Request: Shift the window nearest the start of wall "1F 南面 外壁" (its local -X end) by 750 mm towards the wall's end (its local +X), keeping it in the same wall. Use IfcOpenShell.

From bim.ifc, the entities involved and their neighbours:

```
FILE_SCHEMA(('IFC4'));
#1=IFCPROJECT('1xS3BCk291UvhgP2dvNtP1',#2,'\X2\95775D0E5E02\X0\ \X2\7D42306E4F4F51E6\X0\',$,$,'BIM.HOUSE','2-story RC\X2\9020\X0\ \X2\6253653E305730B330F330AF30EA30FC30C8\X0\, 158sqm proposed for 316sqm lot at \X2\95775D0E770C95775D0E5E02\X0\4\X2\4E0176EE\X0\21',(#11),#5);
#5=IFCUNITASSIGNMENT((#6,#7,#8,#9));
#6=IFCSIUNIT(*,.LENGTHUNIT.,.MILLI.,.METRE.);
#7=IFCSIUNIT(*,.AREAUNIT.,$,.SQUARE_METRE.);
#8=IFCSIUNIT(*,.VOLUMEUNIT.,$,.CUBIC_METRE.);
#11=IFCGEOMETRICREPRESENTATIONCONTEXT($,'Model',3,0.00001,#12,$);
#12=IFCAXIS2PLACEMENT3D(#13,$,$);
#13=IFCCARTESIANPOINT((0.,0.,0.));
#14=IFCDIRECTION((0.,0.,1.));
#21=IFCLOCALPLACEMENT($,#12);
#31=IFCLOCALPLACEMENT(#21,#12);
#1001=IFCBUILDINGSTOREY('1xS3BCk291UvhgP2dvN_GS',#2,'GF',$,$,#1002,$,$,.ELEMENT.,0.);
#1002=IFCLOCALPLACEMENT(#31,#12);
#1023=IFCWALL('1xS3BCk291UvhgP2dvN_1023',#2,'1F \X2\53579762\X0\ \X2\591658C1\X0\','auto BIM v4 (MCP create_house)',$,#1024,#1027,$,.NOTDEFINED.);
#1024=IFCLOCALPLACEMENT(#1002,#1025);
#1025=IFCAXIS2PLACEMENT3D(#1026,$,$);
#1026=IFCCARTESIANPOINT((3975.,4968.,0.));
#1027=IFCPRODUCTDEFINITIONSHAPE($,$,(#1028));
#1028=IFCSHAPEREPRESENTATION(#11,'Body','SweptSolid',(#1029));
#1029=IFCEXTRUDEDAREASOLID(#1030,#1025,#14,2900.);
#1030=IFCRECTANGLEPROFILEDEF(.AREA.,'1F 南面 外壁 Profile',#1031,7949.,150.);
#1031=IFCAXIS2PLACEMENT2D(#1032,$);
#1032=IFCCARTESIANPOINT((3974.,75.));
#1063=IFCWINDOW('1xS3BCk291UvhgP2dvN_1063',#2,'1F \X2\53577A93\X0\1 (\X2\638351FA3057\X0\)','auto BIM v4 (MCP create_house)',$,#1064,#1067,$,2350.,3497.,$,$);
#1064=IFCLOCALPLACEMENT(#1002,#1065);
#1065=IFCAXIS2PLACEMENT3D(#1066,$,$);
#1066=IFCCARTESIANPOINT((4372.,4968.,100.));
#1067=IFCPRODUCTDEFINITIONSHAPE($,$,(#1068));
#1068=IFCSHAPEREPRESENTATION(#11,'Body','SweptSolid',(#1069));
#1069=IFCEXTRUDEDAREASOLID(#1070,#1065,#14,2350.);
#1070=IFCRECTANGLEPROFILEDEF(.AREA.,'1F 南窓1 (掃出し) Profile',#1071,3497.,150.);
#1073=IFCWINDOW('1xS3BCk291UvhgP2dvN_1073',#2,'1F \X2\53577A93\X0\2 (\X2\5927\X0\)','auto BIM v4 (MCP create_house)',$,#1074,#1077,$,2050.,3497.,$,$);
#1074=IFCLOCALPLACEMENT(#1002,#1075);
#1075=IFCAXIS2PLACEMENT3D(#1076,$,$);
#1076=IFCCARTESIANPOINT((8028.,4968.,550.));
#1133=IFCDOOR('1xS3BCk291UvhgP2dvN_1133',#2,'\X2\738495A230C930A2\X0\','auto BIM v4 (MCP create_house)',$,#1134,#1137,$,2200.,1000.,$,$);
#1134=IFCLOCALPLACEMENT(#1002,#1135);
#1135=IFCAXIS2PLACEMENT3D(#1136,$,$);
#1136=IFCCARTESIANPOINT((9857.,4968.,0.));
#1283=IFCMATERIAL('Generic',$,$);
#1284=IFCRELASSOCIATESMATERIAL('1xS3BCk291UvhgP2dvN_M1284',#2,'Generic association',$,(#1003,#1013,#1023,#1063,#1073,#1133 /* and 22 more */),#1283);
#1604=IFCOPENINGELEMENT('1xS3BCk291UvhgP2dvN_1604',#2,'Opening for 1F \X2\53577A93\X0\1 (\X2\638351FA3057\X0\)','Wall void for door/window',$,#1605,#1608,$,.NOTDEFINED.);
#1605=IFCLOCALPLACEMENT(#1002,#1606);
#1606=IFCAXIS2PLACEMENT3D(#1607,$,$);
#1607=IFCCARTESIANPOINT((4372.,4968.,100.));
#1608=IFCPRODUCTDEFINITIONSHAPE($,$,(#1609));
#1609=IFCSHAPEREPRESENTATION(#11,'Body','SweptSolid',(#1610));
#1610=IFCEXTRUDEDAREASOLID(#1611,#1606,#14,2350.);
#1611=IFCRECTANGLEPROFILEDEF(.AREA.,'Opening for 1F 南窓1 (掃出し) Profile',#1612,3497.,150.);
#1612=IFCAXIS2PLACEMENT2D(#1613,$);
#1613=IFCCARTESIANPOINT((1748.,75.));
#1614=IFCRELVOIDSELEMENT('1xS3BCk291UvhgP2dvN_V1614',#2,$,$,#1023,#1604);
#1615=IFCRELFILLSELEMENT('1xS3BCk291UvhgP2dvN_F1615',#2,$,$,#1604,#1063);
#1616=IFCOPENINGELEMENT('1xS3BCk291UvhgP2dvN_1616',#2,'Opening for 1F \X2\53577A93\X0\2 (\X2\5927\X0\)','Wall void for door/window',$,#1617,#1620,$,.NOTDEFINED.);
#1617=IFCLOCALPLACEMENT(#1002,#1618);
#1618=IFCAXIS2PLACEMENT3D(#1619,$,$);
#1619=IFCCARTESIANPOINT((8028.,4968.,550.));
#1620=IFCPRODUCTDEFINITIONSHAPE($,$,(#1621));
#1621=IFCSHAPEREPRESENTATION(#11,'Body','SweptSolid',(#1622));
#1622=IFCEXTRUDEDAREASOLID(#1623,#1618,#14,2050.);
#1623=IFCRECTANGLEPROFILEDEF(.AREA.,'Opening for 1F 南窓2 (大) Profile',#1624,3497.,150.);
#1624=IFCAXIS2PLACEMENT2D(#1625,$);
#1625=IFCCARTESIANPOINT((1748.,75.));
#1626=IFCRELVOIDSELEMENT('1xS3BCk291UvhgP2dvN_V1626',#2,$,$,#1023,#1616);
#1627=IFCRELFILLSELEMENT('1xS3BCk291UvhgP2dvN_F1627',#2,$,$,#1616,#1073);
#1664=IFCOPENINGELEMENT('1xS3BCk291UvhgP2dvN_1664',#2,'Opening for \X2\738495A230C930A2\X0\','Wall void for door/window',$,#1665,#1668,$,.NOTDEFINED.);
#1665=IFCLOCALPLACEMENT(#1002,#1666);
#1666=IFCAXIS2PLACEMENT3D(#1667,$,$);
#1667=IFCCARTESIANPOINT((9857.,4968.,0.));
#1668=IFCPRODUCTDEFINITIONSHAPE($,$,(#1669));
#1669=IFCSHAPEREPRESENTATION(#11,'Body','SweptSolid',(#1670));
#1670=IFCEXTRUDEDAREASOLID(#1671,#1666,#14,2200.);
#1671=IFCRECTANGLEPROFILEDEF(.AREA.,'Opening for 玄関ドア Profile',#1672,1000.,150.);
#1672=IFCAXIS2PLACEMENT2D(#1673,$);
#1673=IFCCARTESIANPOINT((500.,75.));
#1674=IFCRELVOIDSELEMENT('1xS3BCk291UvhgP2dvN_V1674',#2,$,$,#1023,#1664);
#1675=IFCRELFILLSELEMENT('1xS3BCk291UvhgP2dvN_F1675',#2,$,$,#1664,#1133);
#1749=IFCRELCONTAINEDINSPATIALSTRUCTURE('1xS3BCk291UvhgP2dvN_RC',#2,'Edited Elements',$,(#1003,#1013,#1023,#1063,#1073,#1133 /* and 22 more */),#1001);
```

```python
import ifcopenshell
import ifcopenshell.api.geometry
import ifcopenshell.util.placement
import ifcopenshell.util.unit

model = ifcopenshell.open("bim.ifc")
unit_scale = ifcopenshell.util.unit.calculate_unit_scale(model)

window = model.by_guid("1xS3BCk291UvhgP2dvN_1063")
opening = window.FillsVoids[0].RelatingOpeningElement
wall = opening.VoidsElements[0].RelatingBuildingElement

wall_matrix = ifcopenshell.util.placement.get_local_placement(wall.ObjectPlacement)
shift = wall_matrix[:3, 0] * 0.75 / unit_scale
before = ifcopenshell.util.placement.get_local_placement(window.ObjectPlacement)[:3, 3].copy()

# The window is not placed relative to its opening, so move both.
for product in (opening, window):
    matrix = ifcopenshell.util.placement.get_local_placement(product.ObjectPlacement)
    matrix[:3, 3] += shift
    ifcopenshell.api.geometry.edit_object_placement(model, product=product, matrix=matrix, is_si=False)

after = ifcopenshell.util.placement.get_local_placement(window.ObjectPlacement)[:3, 3]
print("window moved by", (after - before).round(3) + 0.0)

model.write("bim_rev.ifc")
```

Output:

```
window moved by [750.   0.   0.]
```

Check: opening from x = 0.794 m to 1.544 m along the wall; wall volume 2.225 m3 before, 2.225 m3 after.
